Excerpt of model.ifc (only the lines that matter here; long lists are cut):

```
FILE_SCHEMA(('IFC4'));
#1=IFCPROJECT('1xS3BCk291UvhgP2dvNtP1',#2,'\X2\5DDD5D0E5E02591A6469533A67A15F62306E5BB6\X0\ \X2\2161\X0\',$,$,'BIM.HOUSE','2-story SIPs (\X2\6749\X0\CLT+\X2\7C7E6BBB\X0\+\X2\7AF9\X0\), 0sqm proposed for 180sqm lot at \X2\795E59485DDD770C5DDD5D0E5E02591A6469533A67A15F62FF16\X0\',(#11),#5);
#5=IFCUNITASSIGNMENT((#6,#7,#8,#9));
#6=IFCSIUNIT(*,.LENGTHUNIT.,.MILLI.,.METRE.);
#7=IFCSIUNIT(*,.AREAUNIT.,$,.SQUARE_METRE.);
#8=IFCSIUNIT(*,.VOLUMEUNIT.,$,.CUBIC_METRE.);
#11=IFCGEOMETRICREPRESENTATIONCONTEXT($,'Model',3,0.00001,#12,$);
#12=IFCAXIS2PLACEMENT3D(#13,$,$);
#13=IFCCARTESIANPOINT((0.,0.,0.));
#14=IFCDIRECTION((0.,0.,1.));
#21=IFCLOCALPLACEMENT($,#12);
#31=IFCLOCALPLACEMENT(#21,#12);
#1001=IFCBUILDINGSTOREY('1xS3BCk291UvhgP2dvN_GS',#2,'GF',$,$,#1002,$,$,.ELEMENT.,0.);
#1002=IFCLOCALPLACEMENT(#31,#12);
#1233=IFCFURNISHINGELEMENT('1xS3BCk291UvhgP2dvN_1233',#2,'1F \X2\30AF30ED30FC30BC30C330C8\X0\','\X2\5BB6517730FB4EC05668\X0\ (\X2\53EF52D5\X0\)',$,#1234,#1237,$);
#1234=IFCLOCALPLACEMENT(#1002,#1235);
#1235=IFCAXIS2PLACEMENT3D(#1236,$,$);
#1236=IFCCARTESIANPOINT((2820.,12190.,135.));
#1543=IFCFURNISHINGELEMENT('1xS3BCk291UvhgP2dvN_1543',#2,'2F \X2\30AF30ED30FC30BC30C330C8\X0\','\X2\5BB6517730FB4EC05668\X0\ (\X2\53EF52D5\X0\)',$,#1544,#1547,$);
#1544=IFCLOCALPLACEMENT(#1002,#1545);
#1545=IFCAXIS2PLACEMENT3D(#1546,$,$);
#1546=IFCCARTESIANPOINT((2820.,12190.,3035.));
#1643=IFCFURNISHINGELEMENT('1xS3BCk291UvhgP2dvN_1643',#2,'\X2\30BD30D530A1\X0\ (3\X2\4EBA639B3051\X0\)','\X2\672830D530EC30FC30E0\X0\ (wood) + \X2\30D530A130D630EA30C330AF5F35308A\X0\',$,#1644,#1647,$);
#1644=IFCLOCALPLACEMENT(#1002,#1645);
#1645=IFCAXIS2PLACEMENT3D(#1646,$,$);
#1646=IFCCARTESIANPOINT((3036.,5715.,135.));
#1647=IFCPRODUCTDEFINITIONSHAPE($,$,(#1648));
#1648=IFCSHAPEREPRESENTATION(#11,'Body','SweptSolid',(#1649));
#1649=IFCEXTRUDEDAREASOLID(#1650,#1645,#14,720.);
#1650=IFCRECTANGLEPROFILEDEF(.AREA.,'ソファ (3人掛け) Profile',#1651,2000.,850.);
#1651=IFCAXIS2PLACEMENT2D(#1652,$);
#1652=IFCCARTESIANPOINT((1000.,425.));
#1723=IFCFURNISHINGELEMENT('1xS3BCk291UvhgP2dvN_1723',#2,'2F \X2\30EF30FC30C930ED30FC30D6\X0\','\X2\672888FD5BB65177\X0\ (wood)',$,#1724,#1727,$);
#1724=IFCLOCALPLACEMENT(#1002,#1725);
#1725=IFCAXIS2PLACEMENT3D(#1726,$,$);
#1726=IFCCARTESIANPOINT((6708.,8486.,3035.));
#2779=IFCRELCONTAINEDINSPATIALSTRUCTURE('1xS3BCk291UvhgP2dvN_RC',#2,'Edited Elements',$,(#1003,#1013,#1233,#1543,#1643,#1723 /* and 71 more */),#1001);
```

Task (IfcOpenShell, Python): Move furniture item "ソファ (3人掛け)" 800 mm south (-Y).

```python
import ifcopenshell
import ifcopenshell.api.geometry
import ifcopenshell.util.placement
import ifcopenshell.util.unit

model = ifcopenshell.open("model.ifc")
unit_scale = ifcopenshell.util.unit.calculate_unit_scale(model)

item = model.by_guid("1xS3BCk291UvhgP2dvN_1643")
matrix = ifcopenshell.util.placement.get_local_placement(item.ObjectPlacement)
matrix[1, 3] -= 0.8 / unit_scale
ifcopenshell.api.geometry.edit_object_placement(model, product=item, matrix=matrix, is_si=False)

print(ifcopenshell.util.placement.get_local_placement(item.ObjectPlacement).round(3) + 0.0)

model.write("model_rev.ifc")
```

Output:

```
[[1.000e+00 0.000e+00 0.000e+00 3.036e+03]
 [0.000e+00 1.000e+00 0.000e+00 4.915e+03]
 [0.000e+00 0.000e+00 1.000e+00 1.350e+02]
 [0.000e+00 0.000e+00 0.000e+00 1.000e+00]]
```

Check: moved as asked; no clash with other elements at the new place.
